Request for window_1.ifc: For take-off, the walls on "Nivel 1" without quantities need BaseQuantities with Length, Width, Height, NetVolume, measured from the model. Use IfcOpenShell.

First a look at what the model holds.

```python
import ifcopenshell
import ifcopenshell.util.element
import ifcopenshell.util.unit

model = ifcopenshell.open("window_1.ifc")
print(model.schema)
for unit_type in ("LENGTHUNIT", "AREAUNIT", "VOLUMEUNIT"):
    print(unit_type, ifcopenshell.util.unit.calculate_unit_scale(model, unit_type))
storey = next(s for s in model.by_type("IfcBuildingStorey") if s.Name == "Nivel 1")
walls = [e for e in ifcopenshell.util.element.get_decomposition(storey) if e.is_a("IfcWall")]
for e in sorted(walls, key=lambda e: e.id()):
    print(e.id(), e.is_a(), e.Name, list(ifcopenshell.util.element.get_psets(e, qtos_only=True)), sep=" | ")
```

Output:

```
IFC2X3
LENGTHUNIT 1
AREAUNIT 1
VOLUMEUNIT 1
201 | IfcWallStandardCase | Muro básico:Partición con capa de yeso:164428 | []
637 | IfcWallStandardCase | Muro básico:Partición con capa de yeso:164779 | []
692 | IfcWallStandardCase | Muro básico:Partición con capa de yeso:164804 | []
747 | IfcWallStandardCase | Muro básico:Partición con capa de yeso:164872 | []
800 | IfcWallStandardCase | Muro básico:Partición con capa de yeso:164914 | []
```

```python
import ifcopenshell
import ifcopenshell.api.pset
import ifcopenshell.geom
import ifcopenshell.util.element
import ifcopenshell.util.shape
import ifcopenshell.util.unit

model = ifcopenshell.open("window_1.ifc")
unit_scale = ifcopenshell.util.unit.calculate_unit_scale(model)
volume_scale = ifcopenshell.util.unit.calculate_unit_scale(model, "VOLUMEUNIT")
settings = ifcopenshell.geom.settings()

storey = next(s for s in model.by_type("IfcBuildingStorey") if s.Name == "Nivel 1")
walls = [e for e in ifcopenshell.util.element.get_decomposition(storey) if e.is_a("IfcWall")]

for e in sorted(walls, key=lambda e: e.id()):
    if ifcopenshell.util.element.get_psets(e, qtos_only=True, should_inherit=False):
        continue
    # Geometry comes back in metres, in the element's own axes.
    shape = ifcopenshell.geom.create_shape(settings, e)
    values = {
        "Length": ifcopenshell.util.shape.get_x(shape.geometry) / unit_scale,
        "Width": ifcopenshell.util.shape.get_y(shape.geometry) / unit_scale,
        "Height": ifcopenshell.util.shape.get_z(shape.geometry) / unit_scale,
        "NetVolume": ifcopenshell.util.shape.get_volume(shape.geometry) / volume_scale,
    }
    qto = ifcopenshell.api.pset.add_qto(model, product=e, name="BaseQuantities")
    ifcopenshell.api.pset.edit_qto(model, qto=qto, properties=values)
    print(e.id(), {k: round(v, 3) for k, v in values.items()})

model.write("window_1_edited.ifc")
```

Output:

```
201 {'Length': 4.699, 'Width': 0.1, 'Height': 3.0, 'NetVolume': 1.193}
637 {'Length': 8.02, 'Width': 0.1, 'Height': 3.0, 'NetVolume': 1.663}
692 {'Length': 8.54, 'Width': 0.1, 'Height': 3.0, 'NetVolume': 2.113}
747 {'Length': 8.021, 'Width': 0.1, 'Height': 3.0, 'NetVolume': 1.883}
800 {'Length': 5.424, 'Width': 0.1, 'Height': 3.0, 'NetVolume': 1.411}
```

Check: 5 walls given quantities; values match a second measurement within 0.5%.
